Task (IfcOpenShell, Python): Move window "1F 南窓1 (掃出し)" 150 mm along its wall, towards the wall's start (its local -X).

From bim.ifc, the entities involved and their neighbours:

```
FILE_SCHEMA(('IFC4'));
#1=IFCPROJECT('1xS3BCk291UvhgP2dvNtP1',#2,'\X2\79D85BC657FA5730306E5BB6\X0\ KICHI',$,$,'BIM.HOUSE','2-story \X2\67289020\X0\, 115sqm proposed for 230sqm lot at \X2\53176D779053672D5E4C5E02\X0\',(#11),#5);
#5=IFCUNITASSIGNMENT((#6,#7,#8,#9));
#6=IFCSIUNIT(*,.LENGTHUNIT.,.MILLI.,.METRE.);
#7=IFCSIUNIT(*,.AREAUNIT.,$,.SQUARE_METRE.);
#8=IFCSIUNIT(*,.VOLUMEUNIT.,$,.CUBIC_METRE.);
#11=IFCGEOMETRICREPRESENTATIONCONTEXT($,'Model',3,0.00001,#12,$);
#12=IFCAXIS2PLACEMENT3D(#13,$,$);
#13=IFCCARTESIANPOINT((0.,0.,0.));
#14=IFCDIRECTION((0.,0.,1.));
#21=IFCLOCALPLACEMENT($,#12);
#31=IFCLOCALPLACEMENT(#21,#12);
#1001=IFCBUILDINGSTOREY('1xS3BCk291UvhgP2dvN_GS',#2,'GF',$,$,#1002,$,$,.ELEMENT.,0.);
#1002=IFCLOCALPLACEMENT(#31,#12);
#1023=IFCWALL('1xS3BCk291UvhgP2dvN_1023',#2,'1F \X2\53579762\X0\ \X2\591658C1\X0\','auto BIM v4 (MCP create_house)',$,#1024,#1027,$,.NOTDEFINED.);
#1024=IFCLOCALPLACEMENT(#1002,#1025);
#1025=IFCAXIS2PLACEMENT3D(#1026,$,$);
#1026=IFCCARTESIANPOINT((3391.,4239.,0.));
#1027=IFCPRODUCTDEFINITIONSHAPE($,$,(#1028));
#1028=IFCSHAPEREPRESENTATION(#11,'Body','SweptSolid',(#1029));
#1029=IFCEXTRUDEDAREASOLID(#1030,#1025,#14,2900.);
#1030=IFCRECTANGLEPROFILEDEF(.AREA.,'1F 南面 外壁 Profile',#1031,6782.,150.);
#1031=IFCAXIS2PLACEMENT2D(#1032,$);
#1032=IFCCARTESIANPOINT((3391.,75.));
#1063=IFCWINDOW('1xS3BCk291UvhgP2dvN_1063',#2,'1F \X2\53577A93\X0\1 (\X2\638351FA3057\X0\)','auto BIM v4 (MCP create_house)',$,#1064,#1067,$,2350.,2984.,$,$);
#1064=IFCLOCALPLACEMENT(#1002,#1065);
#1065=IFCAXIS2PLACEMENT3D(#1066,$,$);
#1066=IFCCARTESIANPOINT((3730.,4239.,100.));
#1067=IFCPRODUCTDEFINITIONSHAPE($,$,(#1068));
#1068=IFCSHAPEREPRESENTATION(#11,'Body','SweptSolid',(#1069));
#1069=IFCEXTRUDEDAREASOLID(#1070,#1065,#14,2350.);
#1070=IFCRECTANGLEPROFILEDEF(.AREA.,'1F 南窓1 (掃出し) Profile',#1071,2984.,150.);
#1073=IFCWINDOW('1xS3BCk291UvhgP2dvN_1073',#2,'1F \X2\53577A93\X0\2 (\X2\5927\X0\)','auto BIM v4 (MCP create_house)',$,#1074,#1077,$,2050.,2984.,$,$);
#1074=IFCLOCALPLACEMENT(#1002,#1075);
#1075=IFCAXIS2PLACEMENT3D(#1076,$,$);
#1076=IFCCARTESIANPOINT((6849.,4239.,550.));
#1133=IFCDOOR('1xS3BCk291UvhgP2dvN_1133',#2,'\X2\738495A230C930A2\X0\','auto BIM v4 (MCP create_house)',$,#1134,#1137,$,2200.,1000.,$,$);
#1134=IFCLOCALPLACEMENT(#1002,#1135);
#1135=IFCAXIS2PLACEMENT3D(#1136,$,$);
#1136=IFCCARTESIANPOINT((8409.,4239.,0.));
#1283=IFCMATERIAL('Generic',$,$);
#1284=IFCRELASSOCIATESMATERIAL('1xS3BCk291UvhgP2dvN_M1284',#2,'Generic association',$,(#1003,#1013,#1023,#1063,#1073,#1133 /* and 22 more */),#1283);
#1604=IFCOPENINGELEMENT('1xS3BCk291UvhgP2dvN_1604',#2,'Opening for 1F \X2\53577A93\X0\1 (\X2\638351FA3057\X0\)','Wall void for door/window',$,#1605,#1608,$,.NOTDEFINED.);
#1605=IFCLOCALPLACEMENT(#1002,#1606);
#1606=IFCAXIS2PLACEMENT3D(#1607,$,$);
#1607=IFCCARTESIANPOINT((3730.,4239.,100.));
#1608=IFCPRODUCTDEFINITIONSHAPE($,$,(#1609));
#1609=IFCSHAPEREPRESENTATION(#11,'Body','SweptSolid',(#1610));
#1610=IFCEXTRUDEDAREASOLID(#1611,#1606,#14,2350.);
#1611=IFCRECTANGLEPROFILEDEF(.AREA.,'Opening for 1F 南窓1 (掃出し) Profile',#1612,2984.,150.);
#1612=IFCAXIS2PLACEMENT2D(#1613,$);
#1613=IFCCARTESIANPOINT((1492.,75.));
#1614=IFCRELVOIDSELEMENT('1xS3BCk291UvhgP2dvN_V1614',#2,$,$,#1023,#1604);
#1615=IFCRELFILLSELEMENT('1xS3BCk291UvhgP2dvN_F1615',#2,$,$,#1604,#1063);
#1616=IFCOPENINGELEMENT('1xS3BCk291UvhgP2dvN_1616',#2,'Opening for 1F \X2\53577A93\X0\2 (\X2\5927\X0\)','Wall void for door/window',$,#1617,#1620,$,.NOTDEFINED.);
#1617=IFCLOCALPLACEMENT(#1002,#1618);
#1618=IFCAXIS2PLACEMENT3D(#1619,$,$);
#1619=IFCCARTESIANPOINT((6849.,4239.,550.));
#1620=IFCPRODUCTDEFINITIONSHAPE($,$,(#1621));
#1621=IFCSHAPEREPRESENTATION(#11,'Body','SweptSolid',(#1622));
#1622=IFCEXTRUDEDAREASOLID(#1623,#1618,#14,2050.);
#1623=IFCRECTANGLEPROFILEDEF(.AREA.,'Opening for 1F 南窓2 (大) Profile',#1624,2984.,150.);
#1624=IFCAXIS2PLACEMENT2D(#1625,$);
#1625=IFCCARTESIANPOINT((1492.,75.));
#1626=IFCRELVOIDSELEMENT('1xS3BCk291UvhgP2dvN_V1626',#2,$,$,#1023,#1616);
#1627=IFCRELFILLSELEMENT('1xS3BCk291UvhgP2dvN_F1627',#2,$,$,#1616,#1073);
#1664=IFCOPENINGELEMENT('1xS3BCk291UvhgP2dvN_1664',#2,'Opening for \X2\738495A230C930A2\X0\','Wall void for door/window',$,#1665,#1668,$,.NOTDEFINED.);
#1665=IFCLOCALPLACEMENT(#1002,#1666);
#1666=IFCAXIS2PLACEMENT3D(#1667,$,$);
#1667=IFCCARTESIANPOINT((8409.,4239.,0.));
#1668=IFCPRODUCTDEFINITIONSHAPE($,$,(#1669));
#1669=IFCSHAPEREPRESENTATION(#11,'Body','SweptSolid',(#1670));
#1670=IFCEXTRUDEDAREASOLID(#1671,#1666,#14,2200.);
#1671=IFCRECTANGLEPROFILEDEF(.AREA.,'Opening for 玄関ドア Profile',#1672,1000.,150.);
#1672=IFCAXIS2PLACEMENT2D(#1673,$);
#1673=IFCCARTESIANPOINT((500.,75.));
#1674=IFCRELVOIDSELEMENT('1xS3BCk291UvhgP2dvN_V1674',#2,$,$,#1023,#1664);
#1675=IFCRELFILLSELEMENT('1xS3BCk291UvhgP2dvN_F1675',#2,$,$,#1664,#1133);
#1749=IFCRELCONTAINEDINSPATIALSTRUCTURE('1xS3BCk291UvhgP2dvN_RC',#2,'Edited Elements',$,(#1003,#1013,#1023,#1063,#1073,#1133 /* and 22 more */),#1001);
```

```python
import ifcopenshell
import ifcopenshell.api.geometry
import ifcopenshell.util.placement
import ifcopenshell.util.unit

model = ifcopenshell.open("bim.ifc")
unit_scale = ifcopenshell.util.unit.calculate_unit_scale(model)

window = model.by_guid("1xS3BCk291UvhgP2dvN_1063")
opening = window.FillsVoids[0].RelatingOpeningElement
wall = opening.VoidsElements[0].RelatingBuildingElement

wall_matrix = ifcopenshell.util.placement.get_local_placement(wall.ObjectPlacement)
shift = wall_matrix[:3, 0] * -0.15 / unit_scale
before = ifcopenshell.util.placement.get_local_placement(window.ObjectPlacement)[:3, 3].copy()

# The window is not placed relative to its opening, so move both.
for product in (opening, window):
    matrix = ifcopenshell.util.placement.get_local_placement(product.ObjectPlacement)
    matrix[:3, 3] += shift
    ifcopenshell.api.geometry.edit_object_placement(model, product=product, matrix=matrix, is_si=False)

after = ifcopenshell.util.placement.get_local_placement(window.ObjectPlacement)[:3, 3]
print("window moved by", (after - before).round(3) + 0.0)

model.write("bim-out.ifc")
```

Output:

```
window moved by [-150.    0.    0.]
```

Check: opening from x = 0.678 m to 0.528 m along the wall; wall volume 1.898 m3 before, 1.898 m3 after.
